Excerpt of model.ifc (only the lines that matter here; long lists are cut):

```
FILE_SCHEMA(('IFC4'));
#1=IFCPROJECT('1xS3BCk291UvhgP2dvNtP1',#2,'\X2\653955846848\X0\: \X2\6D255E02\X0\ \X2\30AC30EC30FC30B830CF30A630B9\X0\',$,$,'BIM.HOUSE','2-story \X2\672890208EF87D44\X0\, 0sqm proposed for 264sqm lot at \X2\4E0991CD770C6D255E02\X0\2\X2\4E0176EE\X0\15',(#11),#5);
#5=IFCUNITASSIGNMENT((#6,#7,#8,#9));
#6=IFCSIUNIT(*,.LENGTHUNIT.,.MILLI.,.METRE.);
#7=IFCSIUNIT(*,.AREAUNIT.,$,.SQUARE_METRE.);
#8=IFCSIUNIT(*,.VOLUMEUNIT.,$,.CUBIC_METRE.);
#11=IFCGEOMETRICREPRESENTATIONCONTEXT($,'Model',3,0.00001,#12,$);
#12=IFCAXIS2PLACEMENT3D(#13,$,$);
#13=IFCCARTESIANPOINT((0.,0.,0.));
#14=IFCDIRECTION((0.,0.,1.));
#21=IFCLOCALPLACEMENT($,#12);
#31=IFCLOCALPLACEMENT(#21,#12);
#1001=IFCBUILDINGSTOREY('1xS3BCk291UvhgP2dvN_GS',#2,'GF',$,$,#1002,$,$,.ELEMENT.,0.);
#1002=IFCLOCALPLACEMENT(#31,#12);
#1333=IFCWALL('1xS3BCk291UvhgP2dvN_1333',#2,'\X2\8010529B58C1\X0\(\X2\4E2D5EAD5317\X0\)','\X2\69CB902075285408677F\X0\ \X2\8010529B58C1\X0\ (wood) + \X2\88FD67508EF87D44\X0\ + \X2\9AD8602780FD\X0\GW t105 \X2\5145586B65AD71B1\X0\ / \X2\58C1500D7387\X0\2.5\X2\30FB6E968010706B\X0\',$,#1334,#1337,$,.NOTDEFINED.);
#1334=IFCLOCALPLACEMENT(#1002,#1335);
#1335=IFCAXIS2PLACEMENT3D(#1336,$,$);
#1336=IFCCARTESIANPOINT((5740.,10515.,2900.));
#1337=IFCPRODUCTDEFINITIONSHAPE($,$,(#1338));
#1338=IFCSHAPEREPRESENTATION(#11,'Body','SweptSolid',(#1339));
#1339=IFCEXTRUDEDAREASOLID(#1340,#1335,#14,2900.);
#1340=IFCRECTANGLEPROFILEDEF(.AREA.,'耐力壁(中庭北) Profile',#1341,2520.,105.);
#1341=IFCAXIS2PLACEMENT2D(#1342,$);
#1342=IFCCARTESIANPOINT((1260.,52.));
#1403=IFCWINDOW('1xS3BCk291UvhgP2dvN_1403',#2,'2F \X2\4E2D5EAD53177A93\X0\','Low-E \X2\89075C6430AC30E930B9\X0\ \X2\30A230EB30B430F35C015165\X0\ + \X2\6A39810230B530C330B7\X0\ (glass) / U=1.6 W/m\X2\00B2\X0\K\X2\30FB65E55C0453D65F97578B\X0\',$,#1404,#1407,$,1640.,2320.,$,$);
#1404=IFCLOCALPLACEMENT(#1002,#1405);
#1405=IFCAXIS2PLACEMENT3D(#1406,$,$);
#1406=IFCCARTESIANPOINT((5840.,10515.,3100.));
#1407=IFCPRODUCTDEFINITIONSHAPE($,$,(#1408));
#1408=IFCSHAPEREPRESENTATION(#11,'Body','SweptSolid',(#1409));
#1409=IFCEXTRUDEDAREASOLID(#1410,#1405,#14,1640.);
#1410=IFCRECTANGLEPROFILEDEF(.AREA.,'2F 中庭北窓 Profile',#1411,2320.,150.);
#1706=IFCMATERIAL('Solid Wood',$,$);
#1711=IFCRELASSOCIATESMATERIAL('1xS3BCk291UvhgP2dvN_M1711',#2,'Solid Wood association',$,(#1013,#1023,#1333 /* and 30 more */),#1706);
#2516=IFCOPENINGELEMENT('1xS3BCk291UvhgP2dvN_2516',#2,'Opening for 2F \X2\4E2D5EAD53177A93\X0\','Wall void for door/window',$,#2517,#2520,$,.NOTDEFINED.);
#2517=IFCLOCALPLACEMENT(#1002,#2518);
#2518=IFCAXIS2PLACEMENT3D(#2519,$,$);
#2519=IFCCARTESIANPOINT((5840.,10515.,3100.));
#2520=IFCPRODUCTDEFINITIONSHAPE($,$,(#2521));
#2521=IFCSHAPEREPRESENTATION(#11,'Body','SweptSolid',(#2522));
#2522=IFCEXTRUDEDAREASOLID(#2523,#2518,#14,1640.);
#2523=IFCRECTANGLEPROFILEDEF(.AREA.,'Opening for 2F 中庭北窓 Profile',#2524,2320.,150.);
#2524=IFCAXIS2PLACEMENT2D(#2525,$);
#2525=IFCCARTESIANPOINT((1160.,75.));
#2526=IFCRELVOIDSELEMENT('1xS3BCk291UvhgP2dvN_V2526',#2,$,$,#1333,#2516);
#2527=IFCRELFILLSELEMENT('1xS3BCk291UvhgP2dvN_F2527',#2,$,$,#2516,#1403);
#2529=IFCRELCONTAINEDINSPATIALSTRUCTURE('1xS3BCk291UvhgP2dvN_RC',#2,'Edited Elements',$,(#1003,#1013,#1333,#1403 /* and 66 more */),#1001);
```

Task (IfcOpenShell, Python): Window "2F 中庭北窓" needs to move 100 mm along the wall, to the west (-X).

```python
import ifcopenshell
import ifcopenshell.api.geometry
import ifcopenshell.util.placement

model = ifcopenshell.open("model.ifc")

window = model.by_guid("1xS3BCk291UvhgP2dvN_1403")
opening = window.FillsVoids[0].RelatingOpeningElement
wall = opening.VoidsElements[0].RelatingBuildingElement

wall_matrix = ifcopenshell.util.placement.get_local_placement(wall.ObjectPlacement)
shift = wall_matrix[:3, 0] * -100.0
before = ifcopenshell.util.placement.get_local_placement(window.ObjectPlacement)[:3, 3].copy()

# The window is not placed relative to its opening, so move both.
for product in (opening, window):
    matrix = ifcopenshell.util.placement.get_local_placement(product.ObjectPlacement)
    matrix[:3, 3] += shift
    ifcopenshell.api.geometry.edit_object_placement(model, product=product, matrix=matrix, is_si=False)

after = ifcopenshell.util.placement.get_local_placement(window.ObjectPlacement)[:3, 3]
print("window moved by", (after - before).round(3) + 0.0)

model.write("model-out.ifc")
```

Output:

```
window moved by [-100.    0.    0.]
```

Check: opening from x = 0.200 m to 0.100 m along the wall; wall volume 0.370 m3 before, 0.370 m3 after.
